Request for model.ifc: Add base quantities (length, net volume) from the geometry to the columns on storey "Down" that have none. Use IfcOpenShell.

First a look at what the model holds.

```python
import ifcopenshell
import ifcopenshell.util.element
import ifcopenshell.util.unit

model = ifcopenshell.open("model.ifc")
print(model.schema)
for unit_type in ("LENGTHUNIT", "AREAUNIT", "VOLUMEUNIT"):
    print(unit_type, ifcopenshell.util.unit.calculate_unit_scale(model, unit_type))
storey = next(s for s in model.by_type("IfcBuildingStorey") if s.Name == "Down")
columns = [e for e in ifcopenshell.util.element.get_decomposition(storey) if e.is_a("IfcColumn")]
for e in sorted(columns, key=lambda e: e.id()):
    print(e.id(), e.is_a(), e.Name, list(ifcopenshell.util.element.get_psets(e, qtos_only=True)), sep=" | ")
```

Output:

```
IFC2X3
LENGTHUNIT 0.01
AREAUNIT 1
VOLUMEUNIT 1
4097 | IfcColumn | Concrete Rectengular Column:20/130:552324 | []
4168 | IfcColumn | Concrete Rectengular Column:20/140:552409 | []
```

```python
import ifcopenshell
import ifcopenshell.api.pset
import ifcopenshell.geom
import ifcopenshell.util.element
import ifcopenshell.util.shape
import ifcopenshell.util.unit

model = ifcopenshell.open("model.ifc")
unit_scale = ifcopenshell.util.unit.calculate_unit_scale(model)
volume_scale = ifcopenshell.util.unit.calculate_unit_scale(model, "VOLUMEUNIT")
settings = ifcopenshell.geom.settings()

storey = next(s for s in model.by_type("IfcBuildingStorey") if s.Name == "Down")
columns = [e for e in ifcopenshell.util.element.get_decomposition(storey) if e.is_a("IfcColumn")]

for e in sorted(columns, key=lambda e: e.id()):
    if ifcopenshell.util.element.get_psets(e, qtos_only=True, should_inherit=False):
        continue
    # Geometry comes back in metres, in the element's own axes.
    shape = ifcopenshell.geom.create_shape(settings, e)
    values = {
        "Length": ifcopenshell.util.shape.get_z(shape.geometry) / unit_scale,
        "NetVolume": ifcopenshell.util.shape.get_volume(shape.geometry) / volume_scale,
    }
    qto = ifcopenshell.api.pset.add_qto(model, product=e, name="BaseQuantities")
    ifcopenshell.api.pset.edit_qto(model, qto=qto, properties=values)
    print(e.id(), {k: round(v, 3) for k, v in values.items()})

model.write("model_v2.ifc")
```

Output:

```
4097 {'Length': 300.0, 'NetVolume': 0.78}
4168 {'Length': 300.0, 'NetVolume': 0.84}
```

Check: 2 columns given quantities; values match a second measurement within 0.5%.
